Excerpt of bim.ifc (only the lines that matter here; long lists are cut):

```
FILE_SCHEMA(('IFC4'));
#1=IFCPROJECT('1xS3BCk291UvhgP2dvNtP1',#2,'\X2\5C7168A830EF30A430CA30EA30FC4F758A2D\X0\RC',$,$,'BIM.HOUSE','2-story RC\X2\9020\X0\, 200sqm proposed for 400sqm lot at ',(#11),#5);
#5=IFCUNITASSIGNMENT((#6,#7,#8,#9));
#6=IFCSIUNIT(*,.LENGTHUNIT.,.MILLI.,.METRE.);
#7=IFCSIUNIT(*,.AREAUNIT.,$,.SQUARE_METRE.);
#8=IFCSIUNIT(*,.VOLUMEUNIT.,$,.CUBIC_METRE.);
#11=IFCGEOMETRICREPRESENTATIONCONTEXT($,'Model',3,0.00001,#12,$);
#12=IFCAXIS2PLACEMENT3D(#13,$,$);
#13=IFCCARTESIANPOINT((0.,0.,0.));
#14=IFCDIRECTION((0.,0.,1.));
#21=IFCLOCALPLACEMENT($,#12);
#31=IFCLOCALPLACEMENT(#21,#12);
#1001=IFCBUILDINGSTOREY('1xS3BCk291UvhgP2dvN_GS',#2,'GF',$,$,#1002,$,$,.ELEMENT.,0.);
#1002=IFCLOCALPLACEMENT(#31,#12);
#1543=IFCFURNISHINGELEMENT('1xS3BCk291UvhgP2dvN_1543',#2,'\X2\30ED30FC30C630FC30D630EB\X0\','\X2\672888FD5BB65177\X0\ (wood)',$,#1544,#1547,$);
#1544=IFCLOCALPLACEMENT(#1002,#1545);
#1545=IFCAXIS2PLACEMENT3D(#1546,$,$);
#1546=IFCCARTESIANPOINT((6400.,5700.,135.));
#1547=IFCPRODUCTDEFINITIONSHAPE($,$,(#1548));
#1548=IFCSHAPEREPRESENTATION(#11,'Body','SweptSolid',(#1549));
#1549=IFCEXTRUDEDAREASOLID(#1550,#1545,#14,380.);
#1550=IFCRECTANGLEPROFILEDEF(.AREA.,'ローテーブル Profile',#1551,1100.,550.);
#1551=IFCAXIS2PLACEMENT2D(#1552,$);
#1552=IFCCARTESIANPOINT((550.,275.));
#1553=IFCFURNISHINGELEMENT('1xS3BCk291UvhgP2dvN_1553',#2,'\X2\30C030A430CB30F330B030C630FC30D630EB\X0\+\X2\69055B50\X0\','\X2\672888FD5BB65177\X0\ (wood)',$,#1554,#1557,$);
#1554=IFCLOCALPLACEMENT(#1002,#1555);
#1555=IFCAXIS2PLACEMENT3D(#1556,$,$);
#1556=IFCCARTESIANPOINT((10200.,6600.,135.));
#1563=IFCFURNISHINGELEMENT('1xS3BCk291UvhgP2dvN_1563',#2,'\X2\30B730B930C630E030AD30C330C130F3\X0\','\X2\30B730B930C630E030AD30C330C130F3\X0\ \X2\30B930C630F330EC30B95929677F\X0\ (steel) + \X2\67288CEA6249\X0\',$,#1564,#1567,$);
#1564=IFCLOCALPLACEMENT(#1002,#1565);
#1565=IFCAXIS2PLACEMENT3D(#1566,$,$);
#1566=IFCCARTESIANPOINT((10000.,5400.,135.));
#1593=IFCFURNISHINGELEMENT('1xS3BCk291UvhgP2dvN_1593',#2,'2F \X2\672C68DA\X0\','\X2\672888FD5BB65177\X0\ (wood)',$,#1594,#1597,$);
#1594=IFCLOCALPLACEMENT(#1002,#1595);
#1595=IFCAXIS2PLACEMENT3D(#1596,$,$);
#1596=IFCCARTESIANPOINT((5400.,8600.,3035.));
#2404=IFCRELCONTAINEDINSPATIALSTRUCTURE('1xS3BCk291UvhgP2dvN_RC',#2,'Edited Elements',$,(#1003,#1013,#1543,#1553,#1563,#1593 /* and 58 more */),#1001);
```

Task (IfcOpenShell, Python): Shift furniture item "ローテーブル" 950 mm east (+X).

```python
import ifcopenshell
import ifcopenshell.api.geometry
import ifcopenshell.util.placement
import ifcopenshell.util.unit

model = ifcopenshell.open("bim.ifc")
unit_scale = ifcopenshell.util.unit.calculate_unit_scale(model)

item = model.by_guid("1xS3BCk291UvhgP2dvN_1543")
matrix = ifcopenshell.util.placement.get_local_placement(item.ObjectPlacement)
matrix[0, 3] += 0.95 / unit_scale
ifcopenshell.api.geometry.edit_object_placement(model, product=item, matrix=matrix, is_si=False)

print(ifcopenshell.util.placement.get_local_placement(item.ObjectPlacement).round(3) + 0.0)

model.write("bim_updated.ifc")
```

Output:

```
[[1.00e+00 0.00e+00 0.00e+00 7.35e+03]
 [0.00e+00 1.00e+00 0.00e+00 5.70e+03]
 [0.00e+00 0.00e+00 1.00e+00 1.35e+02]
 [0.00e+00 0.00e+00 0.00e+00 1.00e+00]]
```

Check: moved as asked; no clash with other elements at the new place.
